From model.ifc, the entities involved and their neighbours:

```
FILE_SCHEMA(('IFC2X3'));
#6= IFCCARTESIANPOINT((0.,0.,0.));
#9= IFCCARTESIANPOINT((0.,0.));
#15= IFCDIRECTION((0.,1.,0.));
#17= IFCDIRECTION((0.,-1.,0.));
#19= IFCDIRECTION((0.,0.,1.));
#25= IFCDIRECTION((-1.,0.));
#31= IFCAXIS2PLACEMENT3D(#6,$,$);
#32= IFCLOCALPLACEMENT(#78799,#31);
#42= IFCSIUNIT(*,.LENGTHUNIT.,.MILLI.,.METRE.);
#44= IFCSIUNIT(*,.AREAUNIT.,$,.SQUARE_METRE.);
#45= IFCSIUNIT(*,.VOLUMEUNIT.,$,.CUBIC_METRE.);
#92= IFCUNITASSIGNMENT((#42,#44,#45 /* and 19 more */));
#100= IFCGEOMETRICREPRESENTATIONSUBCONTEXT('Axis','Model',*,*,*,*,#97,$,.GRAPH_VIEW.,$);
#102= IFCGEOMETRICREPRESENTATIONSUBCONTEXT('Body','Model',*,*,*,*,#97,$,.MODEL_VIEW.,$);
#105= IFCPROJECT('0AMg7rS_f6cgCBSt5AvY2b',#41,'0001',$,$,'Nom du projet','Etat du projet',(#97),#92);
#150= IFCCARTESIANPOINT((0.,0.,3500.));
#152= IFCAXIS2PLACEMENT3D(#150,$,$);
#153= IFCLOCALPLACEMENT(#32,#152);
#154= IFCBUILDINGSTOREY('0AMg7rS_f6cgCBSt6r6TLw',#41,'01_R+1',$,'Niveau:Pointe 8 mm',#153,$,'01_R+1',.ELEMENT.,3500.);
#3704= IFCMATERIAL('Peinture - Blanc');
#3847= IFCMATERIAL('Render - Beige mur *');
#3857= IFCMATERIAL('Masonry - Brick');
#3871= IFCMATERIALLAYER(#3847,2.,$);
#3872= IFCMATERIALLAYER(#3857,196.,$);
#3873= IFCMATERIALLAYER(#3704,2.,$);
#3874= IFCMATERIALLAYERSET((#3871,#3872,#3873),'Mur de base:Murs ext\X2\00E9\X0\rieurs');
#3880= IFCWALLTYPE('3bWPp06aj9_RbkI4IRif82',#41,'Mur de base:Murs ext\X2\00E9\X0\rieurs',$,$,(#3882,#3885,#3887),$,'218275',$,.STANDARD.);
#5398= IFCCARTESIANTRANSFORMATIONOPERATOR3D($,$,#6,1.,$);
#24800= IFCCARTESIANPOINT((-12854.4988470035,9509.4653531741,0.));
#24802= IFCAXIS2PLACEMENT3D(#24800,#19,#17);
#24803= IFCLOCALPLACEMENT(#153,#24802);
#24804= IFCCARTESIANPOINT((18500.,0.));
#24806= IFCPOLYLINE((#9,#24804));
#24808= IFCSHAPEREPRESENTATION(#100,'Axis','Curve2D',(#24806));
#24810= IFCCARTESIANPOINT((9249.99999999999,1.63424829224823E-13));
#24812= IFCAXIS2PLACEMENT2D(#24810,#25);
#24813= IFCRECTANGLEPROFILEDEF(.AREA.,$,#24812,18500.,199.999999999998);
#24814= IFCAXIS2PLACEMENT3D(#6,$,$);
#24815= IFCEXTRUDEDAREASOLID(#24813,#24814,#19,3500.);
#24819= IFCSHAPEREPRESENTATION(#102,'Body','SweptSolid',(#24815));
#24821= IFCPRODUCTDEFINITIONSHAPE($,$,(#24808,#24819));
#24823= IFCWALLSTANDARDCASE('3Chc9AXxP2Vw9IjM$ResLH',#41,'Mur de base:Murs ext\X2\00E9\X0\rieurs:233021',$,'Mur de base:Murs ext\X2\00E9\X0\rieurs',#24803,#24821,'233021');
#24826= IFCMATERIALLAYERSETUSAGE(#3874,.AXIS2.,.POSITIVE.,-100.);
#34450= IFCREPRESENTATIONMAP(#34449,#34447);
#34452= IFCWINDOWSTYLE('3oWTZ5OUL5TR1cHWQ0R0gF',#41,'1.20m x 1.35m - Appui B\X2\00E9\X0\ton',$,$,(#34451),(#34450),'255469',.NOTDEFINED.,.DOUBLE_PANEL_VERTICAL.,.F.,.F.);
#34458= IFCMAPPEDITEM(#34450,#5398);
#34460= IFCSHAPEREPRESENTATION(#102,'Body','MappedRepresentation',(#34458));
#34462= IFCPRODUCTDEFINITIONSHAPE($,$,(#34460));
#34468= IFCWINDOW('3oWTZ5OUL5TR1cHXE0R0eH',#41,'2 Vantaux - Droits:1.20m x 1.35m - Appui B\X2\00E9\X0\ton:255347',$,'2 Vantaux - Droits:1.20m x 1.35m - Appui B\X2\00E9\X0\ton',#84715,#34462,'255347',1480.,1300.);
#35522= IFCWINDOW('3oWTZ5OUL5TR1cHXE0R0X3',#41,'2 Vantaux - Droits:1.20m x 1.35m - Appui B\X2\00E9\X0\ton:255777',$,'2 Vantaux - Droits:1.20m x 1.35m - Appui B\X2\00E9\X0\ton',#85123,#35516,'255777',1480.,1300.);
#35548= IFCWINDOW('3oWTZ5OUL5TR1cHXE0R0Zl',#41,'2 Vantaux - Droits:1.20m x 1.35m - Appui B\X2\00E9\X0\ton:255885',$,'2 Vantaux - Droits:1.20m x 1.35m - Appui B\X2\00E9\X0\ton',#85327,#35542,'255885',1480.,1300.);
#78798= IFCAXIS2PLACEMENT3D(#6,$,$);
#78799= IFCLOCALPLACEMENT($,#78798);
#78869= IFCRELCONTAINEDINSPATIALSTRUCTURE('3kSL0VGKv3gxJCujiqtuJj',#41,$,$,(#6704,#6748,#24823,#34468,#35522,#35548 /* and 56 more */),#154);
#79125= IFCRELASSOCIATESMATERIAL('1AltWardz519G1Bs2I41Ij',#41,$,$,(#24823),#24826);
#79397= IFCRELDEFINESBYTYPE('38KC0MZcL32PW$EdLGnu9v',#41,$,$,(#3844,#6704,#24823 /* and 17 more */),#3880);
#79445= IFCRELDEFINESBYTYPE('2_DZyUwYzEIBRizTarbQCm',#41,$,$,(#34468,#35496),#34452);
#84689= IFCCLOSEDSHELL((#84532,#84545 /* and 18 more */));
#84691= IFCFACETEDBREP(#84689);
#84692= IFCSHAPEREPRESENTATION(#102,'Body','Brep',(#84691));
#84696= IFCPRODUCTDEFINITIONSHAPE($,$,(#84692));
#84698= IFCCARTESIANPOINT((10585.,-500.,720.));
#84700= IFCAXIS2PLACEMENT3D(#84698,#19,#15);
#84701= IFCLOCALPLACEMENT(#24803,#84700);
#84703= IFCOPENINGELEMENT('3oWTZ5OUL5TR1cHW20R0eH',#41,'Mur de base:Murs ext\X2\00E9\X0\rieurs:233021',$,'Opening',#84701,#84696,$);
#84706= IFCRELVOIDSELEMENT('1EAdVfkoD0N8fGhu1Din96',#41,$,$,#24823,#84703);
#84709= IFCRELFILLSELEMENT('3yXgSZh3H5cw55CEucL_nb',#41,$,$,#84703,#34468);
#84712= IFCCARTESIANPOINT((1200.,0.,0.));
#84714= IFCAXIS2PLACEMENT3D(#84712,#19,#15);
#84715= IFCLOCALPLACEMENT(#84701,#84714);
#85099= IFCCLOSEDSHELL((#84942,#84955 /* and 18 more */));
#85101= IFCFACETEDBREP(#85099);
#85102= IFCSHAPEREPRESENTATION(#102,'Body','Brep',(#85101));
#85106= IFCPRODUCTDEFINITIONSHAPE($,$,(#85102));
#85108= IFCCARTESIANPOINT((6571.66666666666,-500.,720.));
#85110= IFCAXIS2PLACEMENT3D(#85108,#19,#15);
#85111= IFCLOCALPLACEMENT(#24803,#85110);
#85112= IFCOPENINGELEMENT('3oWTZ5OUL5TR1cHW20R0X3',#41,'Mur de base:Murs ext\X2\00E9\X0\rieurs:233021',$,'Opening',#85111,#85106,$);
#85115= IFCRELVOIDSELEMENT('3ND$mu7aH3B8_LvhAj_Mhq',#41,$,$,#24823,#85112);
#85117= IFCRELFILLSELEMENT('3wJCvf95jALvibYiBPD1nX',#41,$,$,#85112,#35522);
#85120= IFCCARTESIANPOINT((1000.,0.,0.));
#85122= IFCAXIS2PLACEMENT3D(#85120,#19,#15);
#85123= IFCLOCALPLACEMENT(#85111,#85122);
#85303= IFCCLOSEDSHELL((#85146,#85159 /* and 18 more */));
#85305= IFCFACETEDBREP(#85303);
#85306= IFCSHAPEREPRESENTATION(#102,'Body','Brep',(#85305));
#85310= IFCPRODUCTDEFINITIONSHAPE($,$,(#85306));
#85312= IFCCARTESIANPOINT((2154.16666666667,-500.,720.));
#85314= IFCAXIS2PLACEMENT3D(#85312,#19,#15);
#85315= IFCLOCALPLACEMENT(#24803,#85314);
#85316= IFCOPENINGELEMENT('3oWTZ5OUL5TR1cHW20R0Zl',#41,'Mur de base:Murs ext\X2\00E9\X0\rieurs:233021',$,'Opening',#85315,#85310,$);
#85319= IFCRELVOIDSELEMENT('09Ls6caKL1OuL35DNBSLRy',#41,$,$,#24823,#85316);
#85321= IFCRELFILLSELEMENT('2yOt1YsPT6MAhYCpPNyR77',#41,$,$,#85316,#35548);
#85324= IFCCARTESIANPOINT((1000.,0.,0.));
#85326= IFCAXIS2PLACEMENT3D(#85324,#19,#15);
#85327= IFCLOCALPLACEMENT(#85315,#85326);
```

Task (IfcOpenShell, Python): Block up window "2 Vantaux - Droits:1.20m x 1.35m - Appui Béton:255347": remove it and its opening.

```python
import ifcopenshell
import ifcopenshell.api.feature
import ifcopenshell.api.root
import ifcopenshell.geom
import ifcopenshell.util.shape

model = ifcopenshell.open("model.ifc")
settings = ifcopenshell.geom.settings()


def volume(element):
    """Net volume in cubic metres, openings subtracted."""
    shape = ifcopenshell.geom.create_shape(settings, element)
    return ifcopenshell.util.shape.get_volume(shape.geometry)


window = model.by_guid("3oWTZ5OUL5TR1cHXE0R0eH")
opening = window.FillsVoids[0].RelatingOpeningElement
wall = opening.VoidsElements[0].RelatingBuildingElement
before = volume(wall)

ifcopenshell.api.root.remove_product(model, product=window)
ifcopenshell.api.feature.remove_feature(model, feature=opening)

after = volume(wall)

print(f"wall volume {before:.3f} -> {after:.3f} m3")

model.write("model_rev.ifc")
```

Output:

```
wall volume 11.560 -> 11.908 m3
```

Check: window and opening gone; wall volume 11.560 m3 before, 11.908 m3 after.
